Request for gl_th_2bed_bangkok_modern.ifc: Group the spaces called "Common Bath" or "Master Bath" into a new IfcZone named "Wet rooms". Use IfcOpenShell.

First a look at what the model holds.

```python
import ifcopenshell

model = ifcopenshell.open("gl_th_2bed_bangkok_modern.ifc")
print(model.schema)
seen = {}
for space in model.by_type("IfcSpace"):
    seen[space.LongName] = seen.get(space.LongName, 0) + 1
for name, count in sorted(seen.items(), key=str):
    print(count, "x", name)
print("zones:", [z.Name for z in model.by_type("IfcZone")][:20])
```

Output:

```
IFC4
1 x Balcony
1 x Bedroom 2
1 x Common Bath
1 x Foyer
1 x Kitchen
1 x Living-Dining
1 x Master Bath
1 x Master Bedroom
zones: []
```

```python
import ifcopenshell
import ifcopenshell.api.group
import ifcopenshell.api.root

model = ifcopenshell.open("gl_th_2bed_bangkok_modern.ifc")

names = {"Common Bath", "Master Bath"}
spaces = [s for s in model.by_type("IfcSpace") if s.LongName in names]

zone = ifcopenshell.api.root.create_entity(model, ifc_class="IfcZone", name="Wet rooms")
ifcopenshell.api.group.assign_group(model, products=spaces, group=zone)
print(len(spaces), "spaces in", zone.Name)

model.write("gl_th_2bed_bangkok_modern-out.ifc")
```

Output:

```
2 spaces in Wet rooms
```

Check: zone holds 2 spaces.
